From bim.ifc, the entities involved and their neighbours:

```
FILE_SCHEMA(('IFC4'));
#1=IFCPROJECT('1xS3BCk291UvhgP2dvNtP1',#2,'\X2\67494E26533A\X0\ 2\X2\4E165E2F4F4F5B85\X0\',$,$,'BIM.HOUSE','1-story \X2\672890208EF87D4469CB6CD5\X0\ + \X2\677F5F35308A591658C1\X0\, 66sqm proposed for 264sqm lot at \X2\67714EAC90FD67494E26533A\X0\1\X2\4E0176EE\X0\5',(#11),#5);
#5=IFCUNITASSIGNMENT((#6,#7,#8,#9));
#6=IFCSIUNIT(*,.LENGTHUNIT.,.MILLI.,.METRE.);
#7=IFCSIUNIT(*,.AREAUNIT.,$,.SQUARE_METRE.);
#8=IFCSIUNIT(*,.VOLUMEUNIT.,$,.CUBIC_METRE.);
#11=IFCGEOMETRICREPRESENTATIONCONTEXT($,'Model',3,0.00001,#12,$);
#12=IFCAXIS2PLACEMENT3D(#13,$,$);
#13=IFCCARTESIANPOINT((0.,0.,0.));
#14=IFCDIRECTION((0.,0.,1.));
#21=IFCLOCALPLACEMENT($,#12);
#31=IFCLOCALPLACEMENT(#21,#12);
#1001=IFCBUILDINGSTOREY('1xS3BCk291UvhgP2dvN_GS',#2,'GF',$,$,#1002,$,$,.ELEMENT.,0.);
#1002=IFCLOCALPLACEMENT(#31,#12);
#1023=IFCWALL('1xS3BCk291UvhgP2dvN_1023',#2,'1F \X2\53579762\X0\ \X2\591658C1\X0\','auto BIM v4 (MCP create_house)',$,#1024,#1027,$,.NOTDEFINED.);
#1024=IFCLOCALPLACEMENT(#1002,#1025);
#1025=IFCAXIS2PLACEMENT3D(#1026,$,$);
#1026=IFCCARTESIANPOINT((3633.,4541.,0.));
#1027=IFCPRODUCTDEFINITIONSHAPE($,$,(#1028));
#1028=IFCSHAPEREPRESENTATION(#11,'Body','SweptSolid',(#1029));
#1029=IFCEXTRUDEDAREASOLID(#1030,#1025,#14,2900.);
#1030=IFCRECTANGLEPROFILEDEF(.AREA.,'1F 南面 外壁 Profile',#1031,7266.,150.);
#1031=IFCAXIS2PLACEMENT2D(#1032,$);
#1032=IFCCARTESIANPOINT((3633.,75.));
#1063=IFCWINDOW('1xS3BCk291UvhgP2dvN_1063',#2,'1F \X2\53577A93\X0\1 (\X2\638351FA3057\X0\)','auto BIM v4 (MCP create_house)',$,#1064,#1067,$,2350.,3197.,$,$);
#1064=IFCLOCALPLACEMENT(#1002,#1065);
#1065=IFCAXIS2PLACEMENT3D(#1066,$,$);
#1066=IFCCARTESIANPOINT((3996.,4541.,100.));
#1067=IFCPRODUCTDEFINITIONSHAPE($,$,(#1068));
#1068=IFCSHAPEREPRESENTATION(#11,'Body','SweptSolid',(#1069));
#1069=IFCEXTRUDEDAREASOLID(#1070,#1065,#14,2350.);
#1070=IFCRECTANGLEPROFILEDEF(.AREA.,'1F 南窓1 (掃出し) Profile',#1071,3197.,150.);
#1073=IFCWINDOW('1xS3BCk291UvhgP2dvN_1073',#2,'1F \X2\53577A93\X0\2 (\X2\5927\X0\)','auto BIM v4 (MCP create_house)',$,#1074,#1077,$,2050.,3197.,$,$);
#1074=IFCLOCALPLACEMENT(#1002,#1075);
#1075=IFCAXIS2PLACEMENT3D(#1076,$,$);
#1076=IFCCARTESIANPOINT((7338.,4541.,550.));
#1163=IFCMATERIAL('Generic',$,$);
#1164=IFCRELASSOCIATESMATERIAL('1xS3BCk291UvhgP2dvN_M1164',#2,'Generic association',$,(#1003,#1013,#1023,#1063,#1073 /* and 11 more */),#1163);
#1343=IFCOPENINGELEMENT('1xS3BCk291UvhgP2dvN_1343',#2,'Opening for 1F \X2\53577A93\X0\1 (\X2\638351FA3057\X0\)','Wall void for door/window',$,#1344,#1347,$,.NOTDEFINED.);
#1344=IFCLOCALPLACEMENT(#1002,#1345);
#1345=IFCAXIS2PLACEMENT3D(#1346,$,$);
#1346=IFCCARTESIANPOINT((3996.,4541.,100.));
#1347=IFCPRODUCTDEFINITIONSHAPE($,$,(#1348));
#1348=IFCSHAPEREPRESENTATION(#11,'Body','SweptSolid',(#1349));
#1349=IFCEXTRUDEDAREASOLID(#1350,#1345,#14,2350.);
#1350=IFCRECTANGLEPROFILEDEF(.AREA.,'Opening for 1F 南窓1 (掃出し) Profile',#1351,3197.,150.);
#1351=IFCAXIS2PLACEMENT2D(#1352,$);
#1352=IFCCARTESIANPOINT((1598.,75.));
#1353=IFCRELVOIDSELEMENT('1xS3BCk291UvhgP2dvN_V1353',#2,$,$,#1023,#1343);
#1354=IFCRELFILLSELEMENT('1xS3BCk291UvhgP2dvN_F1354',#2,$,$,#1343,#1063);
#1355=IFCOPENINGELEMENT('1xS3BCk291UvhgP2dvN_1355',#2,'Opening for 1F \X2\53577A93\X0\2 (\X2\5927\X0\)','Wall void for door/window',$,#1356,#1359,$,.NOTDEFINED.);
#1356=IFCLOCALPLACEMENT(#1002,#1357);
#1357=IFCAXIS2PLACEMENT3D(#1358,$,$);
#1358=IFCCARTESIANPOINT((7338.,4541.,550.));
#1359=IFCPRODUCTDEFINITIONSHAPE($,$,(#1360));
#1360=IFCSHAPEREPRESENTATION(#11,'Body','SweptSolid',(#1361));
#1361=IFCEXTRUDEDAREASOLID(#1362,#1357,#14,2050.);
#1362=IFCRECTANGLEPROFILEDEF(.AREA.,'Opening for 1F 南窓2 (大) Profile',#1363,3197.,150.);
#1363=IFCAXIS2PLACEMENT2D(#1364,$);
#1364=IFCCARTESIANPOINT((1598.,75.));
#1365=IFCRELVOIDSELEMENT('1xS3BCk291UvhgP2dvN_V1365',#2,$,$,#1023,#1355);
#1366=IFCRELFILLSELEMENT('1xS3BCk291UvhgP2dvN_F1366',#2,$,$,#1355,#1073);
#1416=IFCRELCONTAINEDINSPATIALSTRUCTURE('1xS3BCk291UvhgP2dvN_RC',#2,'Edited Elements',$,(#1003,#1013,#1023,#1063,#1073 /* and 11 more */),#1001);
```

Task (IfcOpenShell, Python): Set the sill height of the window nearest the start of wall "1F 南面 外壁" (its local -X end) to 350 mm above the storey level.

```python
import numpy as np
import ifcopenshell
import ifcopenshell.api.geometry
import ifcopenshell.geom
import ifcopenshell.util.element
import ifcopenshell.util.placement
import ifcopenshell.util.shape
import ifcopenshell.util.unit

model = ifcopenshell.open("bim.ifc")
unit_scale = ifcopenshell.util.unit.calculate_unit_scale(model)

window = model.by_guid("1xS3BCk291UvhgP2dvN_1063")
opening = window.FillsVoids[0].RelatingOpeningElement
storey = ifcopenshell.util.element.get_container(window, ifc_class="IfcBuildingStorey")
level = ifcopenshell.util.placement.get_local_placement(storey.ObjectPlacement)[2, 3]

# The opening's origin need not be at the sill, so measure its lowest point.
shape = ifcopenshell.geom.create_shape(ifcopenshell.geom.settings(), opening)
bottom = ifcopenshell.util.shape.get_shape_bottom_elevation(shape, shape.geometry) / unit_scale
dz = level + 0.35 / unit_scale - bottom

shift = np.array([0.0, 0.0, dz])
# The window is not placed relative to its opening, so move both.
for product in (opening, window):
    matrix = ifcopenshell.util.placement.get_local_placement(product.ObjectPlacement)
    matrix[:3, 3] += shift
    ifcopenshell.api.geometry.edit_object_placement(model, product=product, matrix=matrix, is_si=False)

print(f"moved by {dz * unit_scale:+.3f} m")

model.write("bim_updated.ifc")
```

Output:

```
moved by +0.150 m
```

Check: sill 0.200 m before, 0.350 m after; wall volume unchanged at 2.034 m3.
